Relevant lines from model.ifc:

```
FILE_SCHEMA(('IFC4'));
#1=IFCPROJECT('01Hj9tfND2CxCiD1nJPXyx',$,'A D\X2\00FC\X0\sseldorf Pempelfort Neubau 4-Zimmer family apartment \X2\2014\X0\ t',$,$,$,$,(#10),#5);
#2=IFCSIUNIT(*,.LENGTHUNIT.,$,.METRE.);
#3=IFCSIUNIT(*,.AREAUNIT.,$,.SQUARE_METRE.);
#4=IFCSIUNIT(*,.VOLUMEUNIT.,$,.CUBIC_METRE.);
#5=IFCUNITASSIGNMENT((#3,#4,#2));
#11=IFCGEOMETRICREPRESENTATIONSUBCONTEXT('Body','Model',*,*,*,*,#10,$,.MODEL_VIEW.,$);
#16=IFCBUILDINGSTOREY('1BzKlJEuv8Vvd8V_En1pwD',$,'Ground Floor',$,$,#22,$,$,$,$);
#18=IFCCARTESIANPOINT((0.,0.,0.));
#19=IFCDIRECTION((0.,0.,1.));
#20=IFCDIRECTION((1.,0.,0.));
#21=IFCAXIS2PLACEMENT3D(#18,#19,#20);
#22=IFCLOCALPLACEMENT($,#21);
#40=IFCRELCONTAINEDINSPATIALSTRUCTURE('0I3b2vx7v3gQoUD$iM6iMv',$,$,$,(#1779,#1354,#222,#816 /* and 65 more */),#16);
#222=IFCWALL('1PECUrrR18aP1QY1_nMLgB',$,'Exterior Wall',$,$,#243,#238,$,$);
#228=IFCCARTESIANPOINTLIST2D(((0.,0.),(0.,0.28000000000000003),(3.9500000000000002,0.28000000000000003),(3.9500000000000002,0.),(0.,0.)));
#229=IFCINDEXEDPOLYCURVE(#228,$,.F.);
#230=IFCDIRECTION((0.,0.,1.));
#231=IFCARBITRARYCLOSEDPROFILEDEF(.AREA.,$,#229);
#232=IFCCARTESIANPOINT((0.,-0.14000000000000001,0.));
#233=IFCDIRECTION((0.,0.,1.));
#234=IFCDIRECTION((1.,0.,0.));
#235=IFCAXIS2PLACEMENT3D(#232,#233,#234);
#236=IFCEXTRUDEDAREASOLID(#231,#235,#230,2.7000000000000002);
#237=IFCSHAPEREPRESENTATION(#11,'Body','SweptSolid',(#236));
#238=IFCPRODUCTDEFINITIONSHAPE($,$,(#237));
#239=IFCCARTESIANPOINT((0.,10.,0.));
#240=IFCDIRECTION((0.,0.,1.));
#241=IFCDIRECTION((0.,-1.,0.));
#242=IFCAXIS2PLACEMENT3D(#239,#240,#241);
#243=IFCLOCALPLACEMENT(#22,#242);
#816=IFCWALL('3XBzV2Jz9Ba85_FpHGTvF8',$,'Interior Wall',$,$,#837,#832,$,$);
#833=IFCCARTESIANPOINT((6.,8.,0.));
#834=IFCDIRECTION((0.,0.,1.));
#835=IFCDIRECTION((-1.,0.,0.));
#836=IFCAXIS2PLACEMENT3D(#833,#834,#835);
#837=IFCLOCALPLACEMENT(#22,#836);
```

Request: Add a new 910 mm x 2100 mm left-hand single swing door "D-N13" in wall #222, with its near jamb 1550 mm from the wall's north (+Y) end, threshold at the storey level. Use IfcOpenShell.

```python
import numpy as np
import ifcopenshell
import ifcopenshell.api.feature
import ifcopenshell.api.geometry
import ifcopenshell.api.root
import ifcopenshell.api.spatial
import ifcopenshell.geom
import ifcopenshell.util.element
import ifcopenshell.util.placement
import ifcopenshell.util.representation
import ifcopenshell.util.shape
import ifcopenshell.util.unit

model = ifcopenshell.open("model.ifc")
unit_scale = ifcopenshell.util.unit.calculate_unit_scale(model)
settings = ifcopenshell.geom.settings()


def volume(element):
    """Net volume in cubic metres, openings subtracted."""
    shape = ifcopenshell.geom.create_shape(settings, element)
    return ifcopenshell.util.shape.get_volume(shape.geometry)


wall = model.by_id(222)
storey = ifcopenshell.util.element.get_container(wall, ifc_class="IfcBuildingStorey")
context = ifcopenshell.util.representation.get_context(model, "Model", "Body", "MODEL_VIEW")
before = volume(wall)

width, height, from_end, sill = 0.91, 2.1, 1.55, 0.0  # metres

# The wall runs along its own X axis, and the end named is its -X end.
wall_shape = ifcopenshell.geom.create_shape(settings, wall)
x, y, z = ifcopenshell.util.shape.get_vertices(wall_shape.geometry).T
start = x.min() + from_end
face, thickness = float(y.min()), float(y.max() - y.min())
wall_matrix = ifcopenshell.util.placement.get_local_placement(wall.ObjectPlacement)
level = ifcopenshell.util.placement.get_local_placement(storey.ObjectPlacement)[2, 3]


def in_wall(x, y):
    """Placement at x, y metres in the wall's axes, at sill height."""
    matrix = wall_matrix.copy()
    matrix[:, 3] = wall_matrix @ np.array([x / unit_scale, y / unit_scale, 0.0, 1.0])
    matrix[2, 3] = level + sill / unit_scale
    return matrix


# Opening: a box that overshoots both wall faces by 50 mm.
opening = ifcopenshell.api.root.create_entity(model, ifc_class="IfcOpeningElement", predefined_type="OPENING")
box = ifcopenshell.api.geometry.add_wall_representation(
    model, context=context, length=width, height=height, thickness=thickness + 0.1
)
ifcopenshell.api.geometry.assign_representation(model, product=opening, representation=box)
ifcopenshell.api.geometry.edit_object_placement(model, product=opening, matrix=in_wall(start, face - 0.05), is_si=False)
ifcopenshell.api.feature.add_feature(model, feature=opening, element=wall)

door = ifcopenshell.api.root.create_entity(model, ifc_class="IfcDoor", name="D-N13", predefined_type="DOOR")
door.OverallWidth, door.OverallHeight = width / unit_scale, height / unit_scale
door.OperationType = "SINGLE_SWING_LEFT"
body = ifcopenshell.api.geometry.add_door_representation(
    model,
    context=context,
    overall_width=door.OverallWidth,
    overall_height=door.OverallHeight,
    operation_type="SINGLE_SWING_LEFT",
    lining_properties={"LiningDepth": thickness / unit_scale, "ThresholdDepth": thickness / unit_scale},
)
ifcopenshell.api.geometry.assign_representation(model, product=door, representation=body)
ifcopenshell.api.spatial.assign_container(model, products=[door], relating_structure=storey)
ifcopenshell.api.feature.add_filling(model, opening=opening, element=door)

# The lining spans the wall, so the door starts at the wall face.
ifcopenshell.api.geometry.edit_object_placement(model, product=door, matrix=in_wall(start, face), is_si=False)

after = volume(wall)

print(f"wall volume {before:.3f} -> {after:.3f} m3")

model.write("model_edited.ifc")
```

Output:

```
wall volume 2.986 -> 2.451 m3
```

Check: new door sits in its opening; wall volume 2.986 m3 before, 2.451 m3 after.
